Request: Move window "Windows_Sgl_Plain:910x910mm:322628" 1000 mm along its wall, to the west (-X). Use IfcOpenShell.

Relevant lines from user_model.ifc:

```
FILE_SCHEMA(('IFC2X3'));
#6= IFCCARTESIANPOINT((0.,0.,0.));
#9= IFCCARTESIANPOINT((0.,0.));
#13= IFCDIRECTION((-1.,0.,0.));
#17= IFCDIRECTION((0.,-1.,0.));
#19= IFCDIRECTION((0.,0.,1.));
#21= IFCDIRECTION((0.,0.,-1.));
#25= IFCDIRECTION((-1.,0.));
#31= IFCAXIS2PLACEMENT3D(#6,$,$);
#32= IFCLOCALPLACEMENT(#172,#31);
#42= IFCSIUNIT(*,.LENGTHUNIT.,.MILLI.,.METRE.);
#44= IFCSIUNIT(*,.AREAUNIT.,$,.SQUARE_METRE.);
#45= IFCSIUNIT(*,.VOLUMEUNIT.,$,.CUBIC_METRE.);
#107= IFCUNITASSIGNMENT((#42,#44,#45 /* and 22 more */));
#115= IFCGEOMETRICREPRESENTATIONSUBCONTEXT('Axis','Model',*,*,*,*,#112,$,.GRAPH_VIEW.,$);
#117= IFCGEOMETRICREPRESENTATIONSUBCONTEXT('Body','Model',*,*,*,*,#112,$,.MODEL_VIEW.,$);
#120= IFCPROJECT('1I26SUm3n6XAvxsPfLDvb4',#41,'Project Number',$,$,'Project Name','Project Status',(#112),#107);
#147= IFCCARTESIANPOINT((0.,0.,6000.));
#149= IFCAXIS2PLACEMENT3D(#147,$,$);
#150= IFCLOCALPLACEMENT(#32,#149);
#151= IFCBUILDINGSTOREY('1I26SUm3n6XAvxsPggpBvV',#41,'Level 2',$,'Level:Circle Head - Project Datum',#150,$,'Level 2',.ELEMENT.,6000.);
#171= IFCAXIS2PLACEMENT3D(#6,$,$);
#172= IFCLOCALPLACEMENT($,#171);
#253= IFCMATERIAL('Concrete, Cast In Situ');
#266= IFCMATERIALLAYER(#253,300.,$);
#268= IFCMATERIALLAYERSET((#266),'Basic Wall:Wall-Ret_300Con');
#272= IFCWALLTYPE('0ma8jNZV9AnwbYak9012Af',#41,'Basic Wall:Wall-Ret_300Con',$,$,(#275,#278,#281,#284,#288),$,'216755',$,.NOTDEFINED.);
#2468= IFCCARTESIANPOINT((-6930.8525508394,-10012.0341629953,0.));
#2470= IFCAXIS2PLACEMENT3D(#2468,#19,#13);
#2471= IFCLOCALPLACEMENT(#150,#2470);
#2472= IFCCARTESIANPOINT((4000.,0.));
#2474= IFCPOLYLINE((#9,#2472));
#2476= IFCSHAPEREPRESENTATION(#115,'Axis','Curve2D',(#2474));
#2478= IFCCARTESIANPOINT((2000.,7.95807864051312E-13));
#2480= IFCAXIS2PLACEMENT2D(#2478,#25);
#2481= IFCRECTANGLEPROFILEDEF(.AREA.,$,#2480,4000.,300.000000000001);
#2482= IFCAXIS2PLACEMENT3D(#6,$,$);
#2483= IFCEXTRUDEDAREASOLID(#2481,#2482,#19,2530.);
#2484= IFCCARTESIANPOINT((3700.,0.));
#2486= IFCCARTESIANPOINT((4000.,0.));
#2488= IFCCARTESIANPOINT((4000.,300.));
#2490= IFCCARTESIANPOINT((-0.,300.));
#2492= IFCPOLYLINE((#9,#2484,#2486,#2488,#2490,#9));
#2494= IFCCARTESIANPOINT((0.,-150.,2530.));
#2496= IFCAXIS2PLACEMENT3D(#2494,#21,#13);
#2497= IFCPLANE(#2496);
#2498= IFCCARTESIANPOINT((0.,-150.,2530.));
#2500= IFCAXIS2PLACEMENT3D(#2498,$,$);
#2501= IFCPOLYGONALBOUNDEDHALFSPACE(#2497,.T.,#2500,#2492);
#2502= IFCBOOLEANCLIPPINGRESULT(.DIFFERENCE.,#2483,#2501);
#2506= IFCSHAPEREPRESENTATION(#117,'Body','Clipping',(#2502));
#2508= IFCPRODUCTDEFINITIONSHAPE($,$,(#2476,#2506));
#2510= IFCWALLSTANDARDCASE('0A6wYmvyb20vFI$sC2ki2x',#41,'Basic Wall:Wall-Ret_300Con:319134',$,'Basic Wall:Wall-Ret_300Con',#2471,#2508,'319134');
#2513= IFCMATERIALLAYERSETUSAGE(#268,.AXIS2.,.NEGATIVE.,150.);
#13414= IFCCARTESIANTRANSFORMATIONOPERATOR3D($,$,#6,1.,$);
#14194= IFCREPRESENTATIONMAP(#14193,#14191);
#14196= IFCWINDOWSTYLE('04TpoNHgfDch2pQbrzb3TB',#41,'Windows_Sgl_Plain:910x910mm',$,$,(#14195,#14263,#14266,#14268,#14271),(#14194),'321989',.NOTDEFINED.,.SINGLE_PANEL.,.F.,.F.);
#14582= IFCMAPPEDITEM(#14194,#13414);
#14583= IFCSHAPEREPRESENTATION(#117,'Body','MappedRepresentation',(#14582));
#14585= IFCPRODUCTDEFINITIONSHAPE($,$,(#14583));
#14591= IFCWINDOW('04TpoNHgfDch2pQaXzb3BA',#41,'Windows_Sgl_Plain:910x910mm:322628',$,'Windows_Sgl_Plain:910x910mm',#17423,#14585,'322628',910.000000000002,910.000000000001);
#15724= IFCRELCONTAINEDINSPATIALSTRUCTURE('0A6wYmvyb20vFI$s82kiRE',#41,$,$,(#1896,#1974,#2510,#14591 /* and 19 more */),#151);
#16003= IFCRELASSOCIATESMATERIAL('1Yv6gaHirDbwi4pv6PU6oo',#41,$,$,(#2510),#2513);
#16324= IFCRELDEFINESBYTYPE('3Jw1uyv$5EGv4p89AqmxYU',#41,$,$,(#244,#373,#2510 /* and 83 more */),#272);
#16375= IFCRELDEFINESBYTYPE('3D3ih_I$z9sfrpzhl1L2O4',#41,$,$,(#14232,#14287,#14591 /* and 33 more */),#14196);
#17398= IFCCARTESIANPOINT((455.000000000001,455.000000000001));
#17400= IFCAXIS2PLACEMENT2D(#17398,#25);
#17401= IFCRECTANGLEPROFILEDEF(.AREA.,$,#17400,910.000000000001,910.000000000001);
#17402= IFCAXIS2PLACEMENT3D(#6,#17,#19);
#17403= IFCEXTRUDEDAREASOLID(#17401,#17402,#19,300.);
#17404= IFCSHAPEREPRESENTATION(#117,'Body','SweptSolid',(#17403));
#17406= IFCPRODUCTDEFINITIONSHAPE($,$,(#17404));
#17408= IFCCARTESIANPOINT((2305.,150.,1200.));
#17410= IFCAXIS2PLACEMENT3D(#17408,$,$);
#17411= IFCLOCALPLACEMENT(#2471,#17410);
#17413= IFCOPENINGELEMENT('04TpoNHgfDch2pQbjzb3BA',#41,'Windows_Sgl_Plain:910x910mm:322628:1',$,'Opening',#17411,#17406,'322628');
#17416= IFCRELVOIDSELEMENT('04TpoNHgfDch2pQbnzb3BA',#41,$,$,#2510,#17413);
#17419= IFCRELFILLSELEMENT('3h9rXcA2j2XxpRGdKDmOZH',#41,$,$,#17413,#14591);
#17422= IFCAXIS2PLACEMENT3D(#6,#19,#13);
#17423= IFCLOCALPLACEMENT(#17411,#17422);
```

```python
import ifcopenshell
import ifcopenshell.api.geometry
import ifcopenshell.util.placement
import ifcopenshell.util.unit

model = ifcopenshell.open("user_model.ifc")
unit_scale = ifcopenshell.util.unit.calculate_unit_scale(model)

window = model.by_guid("04TpoNHgfDch2pQaXzb3BA")
opening = window.FillsVoids[0].RelatingOpeningElement
wall = opening.VoidsElements[0].RelatingBuildingElement

wall_matrix = ifcopenshell.util.placement.get_local_placement(wall.ObjectPlacement)
shift = wall_matrix[:3, 0] * 1 / unit_scale
before = ifcopenshell.util.placement.get_local_placement(window.ObjectPlacement)[:3, 3].copy()

# The window is placed relative to its opening, so it follows when the opening moves.
matrix = ifcopenshell.util.placement.get_local_placement(opening.ObjectPlacement)
matrix[:3, 3] += shift
ifcopenshell.api.geometry.edit_object_placement(
    model, product=opening, matrix=matrix, is_si=False, should_transform_children=True
)

after = ifcopenshell.util.placement.get_local_placement(window.ObjectPlacement)[:3, 3]
print("window moved by", (after - before).round(3) + 0.0)

model.write("user_model_v2.ifc")
```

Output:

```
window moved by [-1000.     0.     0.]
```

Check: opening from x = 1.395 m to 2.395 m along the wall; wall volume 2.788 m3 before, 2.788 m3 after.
